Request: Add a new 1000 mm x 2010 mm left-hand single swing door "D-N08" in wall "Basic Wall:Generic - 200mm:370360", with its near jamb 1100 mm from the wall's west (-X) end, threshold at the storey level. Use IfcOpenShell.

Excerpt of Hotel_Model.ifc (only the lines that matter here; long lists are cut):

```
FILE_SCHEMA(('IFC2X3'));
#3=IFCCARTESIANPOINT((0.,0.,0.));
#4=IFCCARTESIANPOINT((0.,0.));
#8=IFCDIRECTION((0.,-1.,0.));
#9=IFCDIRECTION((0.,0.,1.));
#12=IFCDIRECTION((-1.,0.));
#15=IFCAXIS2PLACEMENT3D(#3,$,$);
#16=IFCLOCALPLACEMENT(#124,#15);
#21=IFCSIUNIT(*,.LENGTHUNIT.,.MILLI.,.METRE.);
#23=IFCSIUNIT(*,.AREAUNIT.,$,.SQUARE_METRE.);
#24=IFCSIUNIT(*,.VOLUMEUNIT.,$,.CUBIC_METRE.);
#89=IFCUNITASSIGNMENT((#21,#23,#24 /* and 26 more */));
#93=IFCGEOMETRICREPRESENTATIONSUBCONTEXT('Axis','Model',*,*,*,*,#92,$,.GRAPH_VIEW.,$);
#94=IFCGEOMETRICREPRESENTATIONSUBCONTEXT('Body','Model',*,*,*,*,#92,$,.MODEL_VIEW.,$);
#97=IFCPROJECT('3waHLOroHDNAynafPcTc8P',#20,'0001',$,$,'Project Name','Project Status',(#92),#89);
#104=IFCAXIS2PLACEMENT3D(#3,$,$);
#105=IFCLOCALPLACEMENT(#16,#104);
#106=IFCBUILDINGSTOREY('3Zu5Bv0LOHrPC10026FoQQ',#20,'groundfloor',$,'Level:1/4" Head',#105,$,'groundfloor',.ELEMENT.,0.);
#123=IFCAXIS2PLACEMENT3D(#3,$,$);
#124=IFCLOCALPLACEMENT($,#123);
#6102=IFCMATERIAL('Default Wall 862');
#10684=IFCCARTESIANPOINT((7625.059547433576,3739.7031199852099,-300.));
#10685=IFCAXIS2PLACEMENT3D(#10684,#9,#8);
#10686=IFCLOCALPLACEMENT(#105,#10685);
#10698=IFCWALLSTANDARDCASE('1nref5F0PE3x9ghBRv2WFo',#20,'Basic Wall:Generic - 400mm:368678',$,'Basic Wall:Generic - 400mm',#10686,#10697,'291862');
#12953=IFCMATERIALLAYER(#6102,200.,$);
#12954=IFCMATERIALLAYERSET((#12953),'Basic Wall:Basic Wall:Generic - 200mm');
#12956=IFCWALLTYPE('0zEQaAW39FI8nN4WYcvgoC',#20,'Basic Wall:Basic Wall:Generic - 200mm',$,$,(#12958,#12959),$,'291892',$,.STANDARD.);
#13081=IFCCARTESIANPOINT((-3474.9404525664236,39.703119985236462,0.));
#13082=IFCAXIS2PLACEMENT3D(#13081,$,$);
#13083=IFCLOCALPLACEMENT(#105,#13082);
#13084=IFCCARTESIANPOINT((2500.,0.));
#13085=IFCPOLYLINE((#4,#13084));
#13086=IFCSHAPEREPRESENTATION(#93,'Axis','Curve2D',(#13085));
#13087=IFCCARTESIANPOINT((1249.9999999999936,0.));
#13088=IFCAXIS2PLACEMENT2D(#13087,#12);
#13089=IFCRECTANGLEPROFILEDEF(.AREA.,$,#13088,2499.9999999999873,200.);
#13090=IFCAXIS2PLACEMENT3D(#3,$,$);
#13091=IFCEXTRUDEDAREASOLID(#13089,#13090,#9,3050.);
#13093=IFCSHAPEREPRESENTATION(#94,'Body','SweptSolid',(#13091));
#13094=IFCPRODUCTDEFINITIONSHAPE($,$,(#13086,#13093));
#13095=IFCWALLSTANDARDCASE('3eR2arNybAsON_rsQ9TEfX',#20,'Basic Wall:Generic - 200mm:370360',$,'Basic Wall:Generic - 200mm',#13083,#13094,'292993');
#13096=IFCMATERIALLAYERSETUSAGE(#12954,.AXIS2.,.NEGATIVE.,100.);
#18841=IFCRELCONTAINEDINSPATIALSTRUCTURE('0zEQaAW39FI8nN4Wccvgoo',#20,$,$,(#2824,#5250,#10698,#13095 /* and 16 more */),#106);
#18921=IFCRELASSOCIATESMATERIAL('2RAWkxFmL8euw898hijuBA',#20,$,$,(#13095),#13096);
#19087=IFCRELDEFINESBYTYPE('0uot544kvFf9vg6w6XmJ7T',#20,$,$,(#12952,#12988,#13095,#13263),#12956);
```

```python
import numpy as np
import ifcopenshell
import ifcopenshell.api.feature
import ifcopenshell.api.geometry
import ifcopenshell.api.root
import ifcopenshell.api.spatial
import ifcopenshell.api.type
import ifcopenshell.geom
import ifcopenshell.util.element
import ifcopenshell.util.placement
import ifcopenshell.util.representation
import ifcopenshell.util.shape
import ifcopenshell.util.unit

model = ifcopenshell.open("Hotel_Model.ifc")
unit_scale = ifcopenshell.util.unit.calculate_unit_scale(model)
settings = ifcopenshell.geom.settings()


def volume(element):
    """Net volume in cubic metres, openings subtracted."""
    shape = ifcopenshell.geom.create_shape(settings, element)
    return ifcopenshell.util.shape.get_volume(shape.geometry)


wall = model.by_guid("3eR2arNybAsON_rsQ9TEfX")
storey = ifcopenshell.util.element.get_container(wall, ifc_class="IfcBuildingStorey")
context = ifcopenshell.util.representation.get_context(model, "Model", "Body", "MODEL_VIEW")
before = volume(wall)

width, height, from_end, sill = 1, 2.01, 1.1, 0.0  # metres

# The wall runs along its own X axis, and the end named is its -X end.
wall_shape = ifcopenshell.geom.create_shape(settings, wall)
x, y, z = ifcopenshell.util.shape.get_vertices(wall_shape.geometry).T
start = x.min() + from_end
face, thickness = float(y.min()), float(y.max() - y.min())
wall_matrix = ifcopenshell.util.placement.get_local_placement(wall.ObjectPlacement)
level = ifcopenshell.util.placement.get_local_placement(storey.ObjectPlacement)[2, 3]


def in_wall(x, y):
    """Placement at x, y metres in the wall's axes, at sill height."""
    matrix = wall_matrix.copy()
    matrix[:, 3] = wall_matrix @ np.array([x / unit_scale, y / unit_scale, 0.0, 1.0])
    matrix[2, 3] = level + sill / unit_scale
    return matrix


# Opening: a box that overshoots both wall faces by 50 mm.
opening = ifcopenshell.api.root.create_entity(model, ifc_class="IfcOpeningElement")
box = ifcopenshell.api.geometry.add_wall_representation(
    model, context=context, length=width, height=height, thickness=thickness + 0.1
)
ifcopenshell.api.geometry.assign_representation(model, product=opening, representation=box)
ifcopenshell.api.geometry.edit_object_placement(model, product=opening, matrix=in_wall(start, face - 0.05), is_si=False)
ifcopenshell.api.feature.add_feature(model, feature=opening, element=wall)

door = ifcopenshell.api.root.create_entity(model, ifc_class="IfcDoor", name="D-N08")
door.OverallWidth, door.OverallHeight = width / unit_scale, height / unit_scale
body = ifcopenshell.api.geometry.add_door_representation(
    model,
    context=context,
    overall_width=door.OverallWidth,
    overall_height=door.OverallHeight,
    operation_type="SINGLE_SWING_LEFT",
    lining_properties={"LiningDepth": thickness / unit_scale, "ThresholdDepth": thickness / unit_scale},
)
ifcopenshell.api.geometry.assign_representation(model, product=door, representation=body)
ifcopenshell.api.spatial.assign_container(model, products=[door], relating_structure=storey)
fills = ifcopenshell.api.feature.add_filling(model, opening=opening, element=door)
fills.OwnerHistory = door.OwnerHistory  # required in IFC2X3

# IFC2X3 keeps the operation on the door style.
style = ifcopenshell.api.root.create_entity(model, ifc_class="IfcDoorStyle", name="D-N08")
style.OperationType, style.ConstructionType = "SINGLE_SWING_LEFT", "NOTDEFINED"
style.ParameterTakesPrecedence = style.Sizeable = False
ifcopenshell.api.type.assign_type(model, related_objects=[door], relating_type=style)

# The lining spans the wall, so the door starts at the wall face.
ifcopenshell.api.geometry.edit_object_placement(model, product=door, matrix=in_wall(start, face), is_si=False)

after = volume(wall)

print(f"wall volume {before:.3f} -> {after:.3f} m3")

model.write("Hotel_Model_edited.ifc")
```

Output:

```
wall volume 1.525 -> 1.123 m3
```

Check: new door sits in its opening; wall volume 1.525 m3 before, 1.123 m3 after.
